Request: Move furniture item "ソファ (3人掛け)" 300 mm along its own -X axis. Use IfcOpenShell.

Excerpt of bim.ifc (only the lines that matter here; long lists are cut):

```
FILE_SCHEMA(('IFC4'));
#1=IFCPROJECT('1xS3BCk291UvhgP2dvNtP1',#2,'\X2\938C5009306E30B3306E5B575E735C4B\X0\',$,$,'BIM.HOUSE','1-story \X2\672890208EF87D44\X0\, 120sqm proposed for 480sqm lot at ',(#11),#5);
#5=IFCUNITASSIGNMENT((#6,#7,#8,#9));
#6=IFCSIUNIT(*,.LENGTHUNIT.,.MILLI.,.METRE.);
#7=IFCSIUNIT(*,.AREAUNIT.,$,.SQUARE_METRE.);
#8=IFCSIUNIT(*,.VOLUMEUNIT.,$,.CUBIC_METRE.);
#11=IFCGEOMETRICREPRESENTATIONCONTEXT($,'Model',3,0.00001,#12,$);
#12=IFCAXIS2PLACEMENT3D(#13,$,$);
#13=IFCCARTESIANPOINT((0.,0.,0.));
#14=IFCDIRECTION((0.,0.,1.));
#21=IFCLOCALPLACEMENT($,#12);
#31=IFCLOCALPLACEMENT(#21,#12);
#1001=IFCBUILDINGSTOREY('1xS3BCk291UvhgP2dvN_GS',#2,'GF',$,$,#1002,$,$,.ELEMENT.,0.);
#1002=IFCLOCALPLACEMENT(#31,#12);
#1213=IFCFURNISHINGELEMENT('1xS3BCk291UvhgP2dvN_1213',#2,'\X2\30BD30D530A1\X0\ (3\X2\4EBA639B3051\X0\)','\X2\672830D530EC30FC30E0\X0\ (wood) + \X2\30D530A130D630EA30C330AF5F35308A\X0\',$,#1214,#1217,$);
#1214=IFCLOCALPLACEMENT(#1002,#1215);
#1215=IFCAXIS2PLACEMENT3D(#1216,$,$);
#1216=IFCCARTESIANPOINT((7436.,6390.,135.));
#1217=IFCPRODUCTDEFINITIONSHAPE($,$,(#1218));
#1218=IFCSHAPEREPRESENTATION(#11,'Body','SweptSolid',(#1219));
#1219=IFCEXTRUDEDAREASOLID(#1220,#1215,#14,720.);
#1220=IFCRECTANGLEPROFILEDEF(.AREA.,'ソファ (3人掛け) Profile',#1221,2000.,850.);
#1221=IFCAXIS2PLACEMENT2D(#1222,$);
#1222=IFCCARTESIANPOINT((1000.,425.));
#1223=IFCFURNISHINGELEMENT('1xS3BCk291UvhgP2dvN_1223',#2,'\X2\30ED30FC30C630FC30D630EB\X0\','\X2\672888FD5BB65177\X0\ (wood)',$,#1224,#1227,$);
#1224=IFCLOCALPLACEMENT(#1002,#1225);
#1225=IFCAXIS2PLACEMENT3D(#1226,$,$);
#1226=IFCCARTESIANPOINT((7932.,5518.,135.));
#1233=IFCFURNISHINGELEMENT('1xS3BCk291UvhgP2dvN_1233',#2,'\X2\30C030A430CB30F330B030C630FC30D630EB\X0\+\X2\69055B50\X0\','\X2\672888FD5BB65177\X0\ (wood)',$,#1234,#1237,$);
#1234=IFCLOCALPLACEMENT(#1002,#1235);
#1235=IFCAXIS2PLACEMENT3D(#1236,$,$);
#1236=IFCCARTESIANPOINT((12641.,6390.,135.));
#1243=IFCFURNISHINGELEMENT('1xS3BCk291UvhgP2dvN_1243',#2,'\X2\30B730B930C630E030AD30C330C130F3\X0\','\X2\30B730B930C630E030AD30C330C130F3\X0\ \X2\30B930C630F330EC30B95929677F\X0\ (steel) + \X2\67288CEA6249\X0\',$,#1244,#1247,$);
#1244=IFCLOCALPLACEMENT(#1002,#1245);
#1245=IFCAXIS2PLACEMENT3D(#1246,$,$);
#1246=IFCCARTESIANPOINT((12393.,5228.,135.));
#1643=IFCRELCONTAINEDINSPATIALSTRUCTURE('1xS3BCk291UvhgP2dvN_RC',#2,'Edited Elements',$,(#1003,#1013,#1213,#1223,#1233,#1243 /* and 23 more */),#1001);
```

```python
import ifcopenshell
import ifcopenshell.api.geometry
import ifcopenshell.util.placement

model = ifcopenshell.open("bim.ifc")

item = model.by_id(1213)
matrix = ifcopenshell.util.placement.get_local_placement(item.ObjectPlacement)
matrix[:3, 3] -= matrix[:3, 0] * 300.0
ifcopenshell.api.geometry.edit_object_placement(model, product=item, matrix=matrix, is_si=False)

print(ifcopenshell.util.placement.get_local_placement(item.ObjectPlacement).round(3) + 0.0)

model.write("bim-out.ifc")
```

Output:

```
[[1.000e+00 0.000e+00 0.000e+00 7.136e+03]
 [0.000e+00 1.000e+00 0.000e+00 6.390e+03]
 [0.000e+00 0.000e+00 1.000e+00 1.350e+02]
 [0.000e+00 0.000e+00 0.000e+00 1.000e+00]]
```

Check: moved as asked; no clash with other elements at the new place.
